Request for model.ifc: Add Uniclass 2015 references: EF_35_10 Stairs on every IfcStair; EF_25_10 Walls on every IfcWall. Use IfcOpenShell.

First a look at what the model holds.

```python
import ifcopenshell

model = ifcopenshell.open("model.ifc")
print(model.schema)
print("classifications:", [c.Name for c in model.by_type("IfcClassification")])
for ifc_class in ("IfcDoor", "IfcRoof", "IfcStair", "IfcWall", "IfcWindow"):
    print(ifc_class, len(model.by_type(ifc_class)))
```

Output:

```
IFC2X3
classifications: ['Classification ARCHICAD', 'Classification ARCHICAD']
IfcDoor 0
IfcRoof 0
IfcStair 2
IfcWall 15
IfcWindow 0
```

```python
import ifcopenshell
import ifcopenshell.api.classification

model = ifcopenshell.open("model.ifc")

# IFC2X3 requires Source and Edition and has no link from the project to the system.
system = model.create_entity("IfcClassification", Source="NBS", Edition="2015", Name="Uniclass 2015")

codes = {
    "IfcStair": ("EF_35_10", "Stairs"),
    "IfcWall": ("EF_25_10", "Walls"),
}
for ifc_class, (code, name) in codes.items():
    products = model.by_type(ifc_class)
    ifcopenshell.api.classification.add_reference(
        model, products=products, classification=system, identification=code, name=name
    )
    print(code, len(products))

model.write("model-out.ifc")
```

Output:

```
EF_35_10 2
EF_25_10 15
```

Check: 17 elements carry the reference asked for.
